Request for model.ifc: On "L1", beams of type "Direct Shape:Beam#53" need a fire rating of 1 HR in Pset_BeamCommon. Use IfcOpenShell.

First a look at what the model holds.

```python
import ifcopenshell
import ifcopenshell.util.element

model = ifcopenshell.open("model.ifc")
print(model.schema)
storey = next(s for s in model.by_type("IfcBuildingStorey") if s.Name == "L1")
beams = [e for e in ifcopenshell.util.element.get_decomposition(storey) if e.is_a("IfcBeam")]
seen = {}
for e in beams:
    element_type = ifcopenshell.util.element.get_type(e)
    key = (element_type.Name if element_type != e and element_type else None, ifcopenshell.util.element.get_pset(e, "Pset_BeamCommon", "FireRating"))
    seen[key] = seen.get(key, 0) + 1
for (name, value), count in sorted(seen.items(), key=str):
    print(count, "x", name, "|", value)
```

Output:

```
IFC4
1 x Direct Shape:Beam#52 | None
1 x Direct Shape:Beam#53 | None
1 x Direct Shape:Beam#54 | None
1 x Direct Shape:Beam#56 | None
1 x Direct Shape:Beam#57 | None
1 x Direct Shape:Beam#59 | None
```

```python
import ifcopenshell
import ifcopenshell.api.pset
import ifcopenshell.util.element

model = ifcopenshell.open("model.ifc")

storey = next(s for s in model.by_type("IfcBuildingStorey") if s.Name == "L1")
beams = [e for e in ifcopenshell.util.element.get_decomposition(storey) if e.is_a("IfcBeam")]

count = 0
for e in beams:
    element_type = ifcopenshell.util.element.get_type(e)
    if element_type in (None, e) or element_type.Name != "Direct Shape:Beam#53":
        continue
    # add_pset returns the element's existing set when there is one.
    pset = ifcopenshell.api.pset.add_pset(model, product=e, name="Pset_BeamCommon")
    ifcopenshell.api.pset.edit_pset(model, pset=pset, properties={"FireRating": "1 HR"})
    count += 1

print(count, "beams updated")

model.write("model_updated.ifc")
```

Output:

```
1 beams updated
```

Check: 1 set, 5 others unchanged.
